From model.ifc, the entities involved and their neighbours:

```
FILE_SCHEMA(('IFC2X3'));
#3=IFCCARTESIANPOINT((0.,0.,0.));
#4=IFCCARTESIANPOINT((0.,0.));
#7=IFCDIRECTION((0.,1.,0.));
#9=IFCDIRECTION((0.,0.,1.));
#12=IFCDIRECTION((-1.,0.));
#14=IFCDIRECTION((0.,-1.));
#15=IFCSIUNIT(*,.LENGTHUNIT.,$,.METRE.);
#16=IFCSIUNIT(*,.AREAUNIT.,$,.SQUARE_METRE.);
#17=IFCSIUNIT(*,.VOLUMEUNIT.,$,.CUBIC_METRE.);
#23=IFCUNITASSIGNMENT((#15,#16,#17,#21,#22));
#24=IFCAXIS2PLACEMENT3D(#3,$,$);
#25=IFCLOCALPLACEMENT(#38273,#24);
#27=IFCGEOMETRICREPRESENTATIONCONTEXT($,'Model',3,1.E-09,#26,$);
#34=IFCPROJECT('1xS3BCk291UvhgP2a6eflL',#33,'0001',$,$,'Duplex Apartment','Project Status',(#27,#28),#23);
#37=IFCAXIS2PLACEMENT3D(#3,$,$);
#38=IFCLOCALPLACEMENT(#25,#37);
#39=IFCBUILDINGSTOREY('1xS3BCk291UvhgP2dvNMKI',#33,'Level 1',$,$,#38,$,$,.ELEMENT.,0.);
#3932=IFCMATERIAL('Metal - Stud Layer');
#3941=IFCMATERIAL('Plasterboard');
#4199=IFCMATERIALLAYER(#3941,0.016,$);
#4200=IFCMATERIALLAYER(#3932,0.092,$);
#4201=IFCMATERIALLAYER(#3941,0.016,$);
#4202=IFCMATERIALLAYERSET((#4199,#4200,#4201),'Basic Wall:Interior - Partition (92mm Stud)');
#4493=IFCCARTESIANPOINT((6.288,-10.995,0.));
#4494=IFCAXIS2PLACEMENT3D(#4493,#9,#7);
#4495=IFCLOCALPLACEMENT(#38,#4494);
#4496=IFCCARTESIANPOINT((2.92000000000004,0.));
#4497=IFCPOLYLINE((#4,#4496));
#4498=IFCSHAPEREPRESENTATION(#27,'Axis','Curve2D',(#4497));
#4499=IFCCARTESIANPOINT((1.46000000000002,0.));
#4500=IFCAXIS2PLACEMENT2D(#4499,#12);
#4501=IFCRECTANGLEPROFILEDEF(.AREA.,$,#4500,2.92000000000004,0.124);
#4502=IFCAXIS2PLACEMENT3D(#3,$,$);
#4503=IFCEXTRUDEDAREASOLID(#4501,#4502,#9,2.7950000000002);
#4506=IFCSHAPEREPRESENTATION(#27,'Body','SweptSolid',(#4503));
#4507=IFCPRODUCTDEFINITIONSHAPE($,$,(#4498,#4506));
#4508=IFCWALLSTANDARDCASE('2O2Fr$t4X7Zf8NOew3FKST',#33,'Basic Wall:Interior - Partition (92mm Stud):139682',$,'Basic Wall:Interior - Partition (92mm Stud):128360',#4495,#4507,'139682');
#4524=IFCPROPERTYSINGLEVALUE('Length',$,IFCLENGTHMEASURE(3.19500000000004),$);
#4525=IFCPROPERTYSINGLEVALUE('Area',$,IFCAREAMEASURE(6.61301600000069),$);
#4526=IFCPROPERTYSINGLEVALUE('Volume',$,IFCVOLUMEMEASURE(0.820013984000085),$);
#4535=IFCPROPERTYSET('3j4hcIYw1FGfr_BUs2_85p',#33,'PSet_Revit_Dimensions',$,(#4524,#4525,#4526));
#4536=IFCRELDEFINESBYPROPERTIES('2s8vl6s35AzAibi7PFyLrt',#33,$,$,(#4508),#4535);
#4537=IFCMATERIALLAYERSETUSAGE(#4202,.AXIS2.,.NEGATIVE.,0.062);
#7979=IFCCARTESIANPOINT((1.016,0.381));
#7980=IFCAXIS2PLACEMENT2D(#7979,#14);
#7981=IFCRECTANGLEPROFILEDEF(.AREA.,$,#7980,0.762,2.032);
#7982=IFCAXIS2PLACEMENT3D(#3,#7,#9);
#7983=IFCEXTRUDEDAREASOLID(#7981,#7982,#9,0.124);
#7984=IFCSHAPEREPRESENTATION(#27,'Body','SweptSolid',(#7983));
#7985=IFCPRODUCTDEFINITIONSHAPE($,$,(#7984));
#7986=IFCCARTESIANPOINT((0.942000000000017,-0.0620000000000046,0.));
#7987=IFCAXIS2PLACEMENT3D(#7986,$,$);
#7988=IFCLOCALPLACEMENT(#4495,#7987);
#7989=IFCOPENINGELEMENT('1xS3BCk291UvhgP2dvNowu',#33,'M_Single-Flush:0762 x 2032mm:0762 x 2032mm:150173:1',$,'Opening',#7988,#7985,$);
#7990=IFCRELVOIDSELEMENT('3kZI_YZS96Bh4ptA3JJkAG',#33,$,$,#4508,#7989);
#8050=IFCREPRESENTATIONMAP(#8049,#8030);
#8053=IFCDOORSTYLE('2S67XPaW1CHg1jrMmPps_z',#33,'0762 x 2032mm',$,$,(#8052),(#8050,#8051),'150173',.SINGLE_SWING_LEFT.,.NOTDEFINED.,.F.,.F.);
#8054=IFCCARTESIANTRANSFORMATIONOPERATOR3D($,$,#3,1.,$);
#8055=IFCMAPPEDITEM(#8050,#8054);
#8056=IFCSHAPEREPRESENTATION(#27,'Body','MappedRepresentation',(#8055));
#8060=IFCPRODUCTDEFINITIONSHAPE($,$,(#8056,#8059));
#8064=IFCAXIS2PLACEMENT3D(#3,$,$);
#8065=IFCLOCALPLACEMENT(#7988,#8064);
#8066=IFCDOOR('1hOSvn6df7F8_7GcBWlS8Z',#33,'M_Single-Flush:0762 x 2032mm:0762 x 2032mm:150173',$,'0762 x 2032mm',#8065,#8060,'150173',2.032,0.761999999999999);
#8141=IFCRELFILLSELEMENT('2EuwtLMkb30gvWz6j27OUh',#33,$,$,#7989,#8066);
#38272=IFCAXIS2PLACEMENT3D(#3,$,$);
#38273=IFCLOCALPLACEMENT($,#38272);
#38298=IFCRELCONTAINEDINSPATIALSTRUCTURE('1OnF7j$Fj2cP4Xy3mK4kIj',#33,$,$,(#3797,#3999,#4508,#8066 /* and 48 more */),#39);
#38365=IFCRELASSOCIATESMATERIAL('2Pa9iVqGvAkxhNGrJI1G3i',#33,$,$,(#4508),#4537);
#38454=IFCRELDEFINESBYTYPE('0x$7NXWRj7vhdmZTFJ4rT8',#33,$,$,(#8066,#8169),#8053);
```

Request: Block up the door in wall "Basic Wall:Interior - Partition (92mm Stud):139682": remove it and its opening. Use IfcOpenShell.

```python
import ifcopenshell
import ifcopenshell.api.feature
import ifcopenshell.api.pset
import ifcopenshell.api.root
import ifcopenshell.geom
import ifcopenshell.util.element
import ifcopenshell.util.shape
import ifcopenshell.util.unit

model = ifcopenshell.open("model.ifc")
area_scale = ifcopenshell.util.unit.calculate_unit_scale(model, "AREAUNIT")
volume_scale = ifcopenshell.util.unit.calculate_unit_scale(model, "VOLUMEUNIT")
settings = ifcopenshell.geom.settings()


def volume(element):
    """Net volume in cubic metres, openings subtracted."""
    shape = ifcopenshell.geom.create_shape(settings, element)
    return ifcopenshell.util.shape.get_volume(shape.geometry)


door = model.by_id(8066)
opening = door.FillsVoids[0].RelatingOpeningElement
wall = opening.VoidsElements[0].RelatingBuildingElement
before = volume(wall)

ifcopenshell.api.root.remove_product(model, product=door)
ifcopenshell.api.feature.remove_feature(model, feature=opening)

after = volume(wall)
thickness = 0.124  # wall thickness in metres

# Update the wall's stored quantities.
pset = model.by_id(ifcopenshell.util.element.get_pset(wall, "PSet_Revit_Dimensions", should_inherit=False)["id"])
ifcopenshell.api.pset.edit_pset(model, pset=pset, properties={
    "Area": model.create_entity("IfcAreaMeasure", after / thickness / area_scale),
    "Volume": model.create_entity("IfcVolumeMeasure", after / volume_scale),
})

print(f"wall volume {before:.3f} -> {after:.3f} m3")

model.write("model-out.ifc")
```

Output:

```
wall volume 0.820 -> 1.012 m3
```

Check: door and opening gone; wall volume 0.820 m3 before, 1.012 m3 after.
